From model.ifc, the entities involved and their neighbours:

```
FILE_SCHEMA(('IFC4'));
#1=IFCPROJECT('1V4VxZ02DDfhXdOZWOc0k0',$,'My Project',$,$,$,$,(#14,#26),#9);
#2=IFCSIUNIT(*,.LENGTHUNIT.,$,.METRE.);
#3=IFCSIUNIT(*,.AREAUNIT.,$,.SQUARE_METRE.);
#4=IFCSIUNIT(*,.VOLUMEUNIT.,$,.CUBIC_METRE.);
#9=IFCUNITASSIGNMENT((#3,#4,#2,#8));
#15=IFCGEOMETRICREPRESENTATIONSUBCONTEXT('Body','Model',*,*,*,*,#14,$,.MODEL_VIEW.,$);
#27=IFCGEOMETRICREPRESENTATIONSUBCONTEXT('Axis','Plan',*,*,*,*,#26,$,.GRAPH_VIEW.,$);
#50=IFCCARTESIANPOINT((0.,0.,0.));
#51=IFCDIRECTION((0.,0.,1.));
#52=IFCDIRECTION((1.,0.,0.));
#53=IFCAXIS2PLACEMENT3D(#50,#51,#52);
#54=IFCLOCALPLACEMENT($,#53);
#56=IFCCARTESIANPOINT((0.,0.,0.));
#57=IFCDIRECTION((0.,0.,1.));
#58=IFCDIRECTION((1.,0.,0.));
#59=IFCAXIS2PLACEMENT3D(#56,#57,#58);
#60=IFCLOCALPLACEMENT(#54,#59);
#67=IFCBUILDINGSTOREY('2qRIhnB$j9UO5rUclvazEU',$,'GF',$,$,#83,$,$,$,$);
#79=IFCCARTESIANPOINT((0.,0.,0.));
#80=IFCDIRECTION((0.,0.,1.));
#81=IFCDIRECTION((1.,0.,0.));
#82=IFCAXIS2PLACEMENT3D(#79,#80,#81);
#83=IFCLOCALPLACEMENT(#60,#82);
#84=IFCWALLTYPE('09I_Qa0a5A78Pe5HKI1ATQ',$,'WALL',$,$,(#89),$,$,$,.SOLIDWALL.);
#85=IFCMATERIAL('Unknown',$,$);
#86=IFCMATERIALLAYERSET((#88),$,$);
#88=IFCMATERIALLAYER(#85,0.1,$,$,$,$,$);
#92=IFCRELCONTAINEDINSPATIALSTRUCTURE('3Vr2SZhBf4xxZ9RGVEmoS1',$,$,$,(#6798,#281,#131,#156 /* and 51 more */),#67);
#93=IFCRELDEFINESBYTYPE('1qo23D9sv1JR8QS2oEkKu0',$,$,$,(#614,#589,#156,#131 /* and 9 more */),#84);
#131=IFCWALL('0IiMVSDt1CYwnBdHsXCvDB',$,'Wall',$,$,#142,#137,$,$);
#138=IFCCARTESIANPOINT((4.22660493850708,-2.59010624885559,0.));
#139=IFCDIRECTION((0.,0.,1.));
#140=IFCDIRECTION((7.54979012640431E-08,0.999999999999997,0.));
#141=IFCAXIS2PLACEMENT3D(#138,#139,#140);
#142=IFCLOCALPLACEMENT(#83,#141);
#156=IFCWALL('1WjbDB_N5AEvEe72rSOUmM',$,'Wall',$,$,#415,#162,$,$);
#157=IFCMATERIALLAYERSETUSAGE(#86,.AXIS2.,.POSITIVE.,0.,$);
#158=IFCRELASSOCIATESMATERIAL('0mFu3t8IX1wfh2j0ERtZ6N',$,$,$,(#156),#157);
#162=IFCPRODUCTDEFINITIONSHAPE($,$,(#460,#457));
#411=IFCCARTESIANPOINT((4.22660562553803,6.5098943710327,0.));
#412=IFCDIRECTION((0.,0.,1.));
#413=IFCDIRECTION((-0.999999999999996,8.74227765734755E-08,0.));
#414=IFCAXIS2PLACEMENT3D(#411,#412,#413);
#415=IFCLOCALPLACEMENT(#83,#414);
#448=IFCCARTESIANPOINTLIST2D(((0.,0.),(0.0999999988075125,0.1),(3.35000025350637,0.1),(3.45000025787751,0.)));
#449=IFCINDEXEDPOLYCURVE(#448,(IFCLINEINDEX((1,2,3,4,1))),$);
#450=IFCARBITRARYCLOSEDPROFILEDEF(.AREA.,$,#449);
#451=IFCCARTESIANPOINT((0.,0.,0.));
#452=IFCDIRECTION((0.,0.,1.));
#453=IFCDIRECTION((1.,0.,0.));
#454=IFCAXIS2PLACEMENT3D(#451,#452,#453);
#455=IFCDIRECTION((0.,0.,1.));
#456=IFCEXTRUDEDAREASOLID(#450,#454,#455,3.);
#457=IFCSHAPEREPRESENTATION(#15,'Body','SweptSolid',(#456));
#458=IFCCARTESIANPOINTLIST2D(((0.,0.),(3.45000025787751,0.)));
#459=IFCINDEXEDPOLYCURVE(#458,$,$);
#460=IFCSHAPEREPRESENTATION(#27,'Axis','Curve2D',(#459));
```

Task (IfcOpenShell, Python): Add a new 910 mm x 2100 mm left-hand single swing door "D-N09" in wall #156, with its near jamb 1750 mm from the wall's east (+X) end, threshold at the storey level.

```python
import numpy as np
import ifcopenshell
import ifcopenshell.api.feature
import ifcopenshell.api.geometry
import ifcopenshell.api.root
import ifcopenshell.api.spatial
import ifcopenshell.geom
import ifcopenshell.util.element
import ifcopenshell.util.placement
import ifcopenshell.util.representation
import ifcopenshell.util.shape
import ifcopenshell.util.unit

model = ifcopenshell.open("model.ifc")
unit_scale = ifcopenshell.util.unit.calculate_unit_scale(model)
settings = ifcopenshell.geom.settings()


def volume(element):
    """Net volume in cubic metres, openings subtracted."""
    shape = ifcopenshell.geom.create_shape(settings, element)
    return ifcopenshell.util.shape.get_volume(shape.geometry)


wall = model.by_guid("1WjbDB_N5AEvEe72rSOUmM")
storey = ifcopenshell.util.element.get_container(wall, ifc_class="IfcBuildingStorey")
context = ifcopenshell.util.representation.get_context(model, "Model", "Body", "MODEL_VIEW")
before = volume(wall)

width, height, from_end, sill = 0.91, 2.1, 1.75, 0.0  # metres

# The wall runs along its own X axis, and the end named is its -X end.
wall_shape = ifcopenshell.geom.create_shape(settings, wall)
x, y, z = ifcopenshell.util.shape.get_vertices(wall_shape.geometry).T
start = x.min() + from_end
face, thickness = float(y.min()), float(y.max() - y.min())
wall_matrix = ifcopenshell.util.placement.get_local_placement(wall.ObjectPlacement)
level = ifcopenshell.util.placement.get_local_placement(storey.ObjectPlacement)[2, 3]


def in_wall(x, y):
    """Placement at x, y metres in the wall's axes, at sill height."""
    matrix = wall_matrix.copy()
    matrix[:, 3] = wall_matrix @ np.array([x / unit_scale, y / unit_scale, 0.0, 1.0])
    matrix[2, 3] = level + sill / unit_scale
    return matrix


# Opening: a box that overshoots both wall faces by 50 mm.
opening = ifcopenshell.api.root.create_entity(model, ifc_class="IfcOpeningElement", predefined_type="OPENING")
box = ifcopenshell.api.geometry.add_wall_representation(
    model, context=context, length=width, height=height, thickness=thickness + 0.1
)
ifcopenshell.api.geometry.assign_representation(model, product=opening, representation=box)
ifcopenshell.api.geometry.edit_object_placement(model, product=opening, matrix=in_wall(start, face - 0.05), is_si=False)
ifcopenshell.api.feature.add_feature(model, feature=opening, element=wall)

door = ifcopenshell.api.root.create_entity(model, ifc_class="IfcDoor", name="D-N09", predefined_type="DOOR")
door.OverallWidth, door.OverallHeight = width / unit_scale, height / unit_scale
door.OperationType = "SINGLE_SWING_LEFT"
body = ifcopenshell.api.geometry.add_door_representation(
    model,
    context=context,
    overall_width=door.OverallWidth,
    overall_height=door.OverallHeight,
    operation_type="SINGLE_SWING_LEFT",
    lining_properties={"LiningDepth": thickness / unit_scale, "ThresholdDepth": thickness / unit_scale},
)
ifcopenshell.api.geometry.assign_representation(model, product=door, representation=body)
ifcopenshell.api.spatial.assign_container(model, products=[door], relating_structure=storey)
ifcopenshell.api.feature.add_filling(model, opening=opening, element=door)

# The lining spans the wall, so the door starts at the wall face.
ifcopenshell.api.geometry.edit_object_placement(model, product=door, matrix=in_wall(start, face), is_si=False)

after = volume(wall)

print(f"wall volume {before:.3f} -> {after:.3f} m3")

model.write("model_rev.ifc")
```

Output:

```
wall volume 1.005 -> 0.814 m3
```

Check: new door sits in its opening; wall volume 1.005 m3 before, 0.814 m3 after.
